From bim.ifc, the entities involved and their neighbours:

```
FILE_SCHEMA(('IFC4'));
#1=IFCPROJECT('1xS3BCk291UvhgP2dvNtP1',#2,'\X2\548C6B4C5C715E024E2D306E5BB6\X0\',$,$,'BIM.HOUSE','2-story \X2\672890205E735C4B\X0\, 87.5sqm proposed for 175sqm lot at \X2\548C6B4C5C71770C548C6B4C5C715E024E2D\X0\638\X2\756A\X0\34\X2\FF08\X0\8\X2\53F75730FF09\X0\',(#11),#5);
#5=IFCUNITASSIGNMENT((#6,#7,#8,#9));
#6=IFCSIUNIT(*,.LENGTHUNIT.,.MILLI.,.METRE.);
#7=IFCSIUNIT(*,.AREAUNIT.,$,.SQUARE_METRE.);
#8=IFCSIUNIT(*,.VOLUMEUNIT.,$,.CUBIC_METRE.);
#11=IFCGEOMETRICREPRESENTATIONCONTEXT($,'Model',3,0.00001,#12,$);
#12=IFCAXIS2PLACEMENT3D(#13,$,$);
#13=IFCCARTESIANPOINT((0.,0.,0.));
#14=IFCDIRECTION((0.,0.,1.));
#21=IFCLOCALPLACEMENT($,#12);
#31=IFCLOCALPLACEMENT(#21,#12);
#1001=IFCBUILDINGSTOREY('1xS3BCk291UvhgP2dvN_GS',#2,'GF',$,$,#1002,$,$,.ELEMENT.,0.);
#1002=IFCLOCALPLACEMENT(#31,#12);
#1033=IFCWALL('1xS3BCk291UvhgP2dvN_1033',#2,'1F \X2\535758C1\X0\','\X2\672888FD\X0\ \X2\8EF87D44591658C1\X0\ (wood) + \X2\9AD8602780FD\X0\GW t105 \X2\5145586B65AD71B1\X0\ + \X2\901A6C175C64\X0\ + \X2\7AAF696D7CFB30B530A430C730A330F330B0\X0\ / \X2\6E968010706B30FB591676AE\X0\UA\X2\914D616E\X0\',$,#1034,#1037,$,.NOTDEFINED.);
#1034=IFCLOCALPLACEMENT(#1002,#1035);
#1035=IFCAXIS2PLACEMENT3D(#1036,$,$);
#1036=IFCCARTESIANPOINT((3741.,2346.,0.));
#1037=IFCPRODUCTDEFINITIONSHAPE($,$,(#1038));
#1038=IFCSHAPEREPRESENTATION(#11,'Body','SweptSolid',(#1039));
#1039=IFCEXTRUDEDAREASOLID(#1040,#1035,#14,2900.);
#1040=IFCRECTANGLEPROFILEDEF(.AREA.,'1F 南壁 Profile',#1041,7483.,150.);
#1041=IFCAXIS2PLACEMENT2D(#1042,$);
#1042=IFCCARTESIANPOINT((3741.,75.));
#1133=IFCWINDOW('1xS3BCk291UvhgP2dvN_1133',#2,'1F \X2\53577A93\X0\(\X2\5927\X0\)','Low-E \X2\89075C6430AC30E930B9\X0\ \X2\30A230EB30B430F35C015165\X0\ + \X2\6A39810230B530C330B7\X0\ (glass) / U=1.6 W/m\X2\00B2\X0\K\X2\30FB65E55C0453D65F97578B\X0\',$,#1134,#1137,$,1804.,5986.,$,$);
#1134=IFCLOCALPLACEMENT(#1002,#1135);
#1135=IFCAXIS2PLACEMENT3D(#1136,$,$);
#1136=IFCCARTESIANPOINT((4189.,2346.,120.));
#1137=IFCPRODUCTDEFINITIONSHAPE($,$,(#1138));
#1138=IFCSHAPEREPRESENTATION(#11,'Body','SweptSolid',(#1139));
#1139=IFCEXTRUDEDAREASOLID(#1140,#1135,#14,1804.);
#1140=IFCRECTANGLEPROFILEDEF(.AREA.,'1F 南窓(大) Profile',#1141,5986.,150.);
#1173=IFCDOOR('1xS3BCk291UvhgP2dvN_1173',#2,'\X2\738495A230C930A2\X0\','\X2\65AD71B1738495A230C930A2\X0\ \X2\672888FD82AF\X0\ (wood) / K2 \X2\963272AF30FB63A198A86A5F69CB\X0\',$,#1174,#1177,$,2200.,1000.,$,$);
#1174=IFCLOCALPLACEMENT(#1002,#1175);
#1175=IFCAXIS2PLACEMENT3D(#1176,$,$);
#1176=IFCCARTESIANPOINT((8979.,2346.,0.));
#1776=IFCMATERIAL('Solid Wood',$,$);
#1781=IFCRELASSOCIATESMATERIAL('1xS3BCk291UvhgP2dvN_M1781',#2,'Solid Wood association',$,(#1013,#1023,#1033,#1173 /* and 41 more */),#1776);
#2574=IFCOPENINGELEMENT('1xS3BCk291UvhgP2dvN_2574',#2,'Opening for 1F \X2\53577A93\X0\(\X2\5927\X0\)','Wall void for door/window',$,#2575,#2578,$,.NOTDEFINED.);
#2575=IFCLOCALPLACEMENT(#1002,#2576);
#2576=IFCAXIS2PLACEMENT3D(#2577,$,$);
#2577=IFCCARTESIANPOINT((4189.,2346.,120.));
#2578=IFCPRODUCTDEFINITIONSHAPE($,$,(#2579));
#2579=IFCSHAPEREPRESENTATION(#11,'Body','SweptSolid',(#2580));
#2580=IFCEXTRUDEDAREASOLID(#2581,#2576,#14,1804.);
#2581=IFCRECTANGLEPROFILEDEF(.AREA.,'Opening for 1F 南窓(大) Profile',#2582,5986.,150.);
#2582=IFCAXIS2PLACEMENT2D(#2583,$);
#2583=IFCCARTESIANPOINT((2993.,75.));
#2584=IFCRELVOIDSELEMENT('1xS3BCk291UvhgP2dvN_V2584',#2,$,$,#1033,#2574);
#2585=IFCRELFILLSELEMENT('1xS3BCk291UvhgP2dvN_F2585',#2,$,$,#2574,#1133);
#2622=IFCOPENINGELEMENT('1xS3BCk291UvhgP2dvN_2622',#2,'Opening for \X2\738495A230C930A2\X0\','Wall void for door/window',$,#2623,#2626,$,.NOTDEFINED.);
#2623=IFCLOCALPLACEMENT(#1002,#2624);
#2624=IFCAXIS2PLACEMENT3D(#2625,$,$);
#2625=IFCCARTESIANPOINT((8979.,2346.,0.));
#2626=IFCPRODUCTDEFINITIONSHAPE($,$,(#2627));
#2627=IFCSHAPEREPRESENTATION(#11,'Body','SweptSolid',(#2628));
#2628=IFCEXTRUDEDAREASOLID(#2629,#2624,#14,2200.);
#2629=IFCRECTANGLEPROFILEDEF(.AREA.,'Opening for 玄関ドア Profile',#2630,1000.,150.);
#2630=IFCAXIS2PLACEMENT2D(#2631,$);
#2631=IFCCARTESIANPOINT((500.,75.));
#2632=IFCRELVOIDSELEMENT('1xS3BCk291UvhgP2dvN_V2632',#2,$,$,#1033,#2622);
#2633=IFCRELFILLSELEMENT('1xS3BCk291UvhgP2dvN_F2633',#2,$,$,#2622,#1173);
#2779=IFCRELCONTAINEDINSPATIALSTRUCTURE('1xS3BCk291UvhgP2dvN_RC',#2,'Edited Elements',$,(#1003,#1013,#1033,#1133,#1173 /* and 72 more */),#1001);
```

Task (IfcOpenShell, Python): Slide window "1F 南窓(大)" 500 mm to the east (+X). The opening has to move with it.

```python
import ifcopenshell
import ifcopenshell.api.geometry
import ifcopenshell.util.placement
import ifcopenshell.util.unit

model = ifcopenshell.open("bim.ifc")
unit_scale = ifcopenshell.util.unit.calculate_unit_scale(model)

window = model.by_guid("1xS3BCk291UvhgP2dvN_1133")
opening = window.FillsVoids[0].RelatingOpeningElement
wall = opening.VoidsElements[0].RelatingBuildingElement

wall_matrix = ifcopenshell.util.placement.get_local_placement(wall.ObjectPlacement)
shift = wall_matrix[:3, 0] * 0.5 / unit_scale
before = ifcopenshell.util.placement.get_local_placement(window.ObjectPlacement)[:3, 3].copy()

# The window is not placed relative to its opening, so move both.
for product in (opening, window):
    matrix = ifcopenshell.util.placement.get_local_placement(product.ObjectPlacement)
    matrix[:3, 3] += shift
    ifcopenshell.api.geometry.edit_object_placement(model, product=product, matrix=matrix, is_si=False)

after = ifcopenshell.util.placement.get_local_placement(window.ObjectPlacement)[:3, 3]
print("window moved by", (after - before).round(3) + 0.0)

model.write("bim_edited.ifc")
```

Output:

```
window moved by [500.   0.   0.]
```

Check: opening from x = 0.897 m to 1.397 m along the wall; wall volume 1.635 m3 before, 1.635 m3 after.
